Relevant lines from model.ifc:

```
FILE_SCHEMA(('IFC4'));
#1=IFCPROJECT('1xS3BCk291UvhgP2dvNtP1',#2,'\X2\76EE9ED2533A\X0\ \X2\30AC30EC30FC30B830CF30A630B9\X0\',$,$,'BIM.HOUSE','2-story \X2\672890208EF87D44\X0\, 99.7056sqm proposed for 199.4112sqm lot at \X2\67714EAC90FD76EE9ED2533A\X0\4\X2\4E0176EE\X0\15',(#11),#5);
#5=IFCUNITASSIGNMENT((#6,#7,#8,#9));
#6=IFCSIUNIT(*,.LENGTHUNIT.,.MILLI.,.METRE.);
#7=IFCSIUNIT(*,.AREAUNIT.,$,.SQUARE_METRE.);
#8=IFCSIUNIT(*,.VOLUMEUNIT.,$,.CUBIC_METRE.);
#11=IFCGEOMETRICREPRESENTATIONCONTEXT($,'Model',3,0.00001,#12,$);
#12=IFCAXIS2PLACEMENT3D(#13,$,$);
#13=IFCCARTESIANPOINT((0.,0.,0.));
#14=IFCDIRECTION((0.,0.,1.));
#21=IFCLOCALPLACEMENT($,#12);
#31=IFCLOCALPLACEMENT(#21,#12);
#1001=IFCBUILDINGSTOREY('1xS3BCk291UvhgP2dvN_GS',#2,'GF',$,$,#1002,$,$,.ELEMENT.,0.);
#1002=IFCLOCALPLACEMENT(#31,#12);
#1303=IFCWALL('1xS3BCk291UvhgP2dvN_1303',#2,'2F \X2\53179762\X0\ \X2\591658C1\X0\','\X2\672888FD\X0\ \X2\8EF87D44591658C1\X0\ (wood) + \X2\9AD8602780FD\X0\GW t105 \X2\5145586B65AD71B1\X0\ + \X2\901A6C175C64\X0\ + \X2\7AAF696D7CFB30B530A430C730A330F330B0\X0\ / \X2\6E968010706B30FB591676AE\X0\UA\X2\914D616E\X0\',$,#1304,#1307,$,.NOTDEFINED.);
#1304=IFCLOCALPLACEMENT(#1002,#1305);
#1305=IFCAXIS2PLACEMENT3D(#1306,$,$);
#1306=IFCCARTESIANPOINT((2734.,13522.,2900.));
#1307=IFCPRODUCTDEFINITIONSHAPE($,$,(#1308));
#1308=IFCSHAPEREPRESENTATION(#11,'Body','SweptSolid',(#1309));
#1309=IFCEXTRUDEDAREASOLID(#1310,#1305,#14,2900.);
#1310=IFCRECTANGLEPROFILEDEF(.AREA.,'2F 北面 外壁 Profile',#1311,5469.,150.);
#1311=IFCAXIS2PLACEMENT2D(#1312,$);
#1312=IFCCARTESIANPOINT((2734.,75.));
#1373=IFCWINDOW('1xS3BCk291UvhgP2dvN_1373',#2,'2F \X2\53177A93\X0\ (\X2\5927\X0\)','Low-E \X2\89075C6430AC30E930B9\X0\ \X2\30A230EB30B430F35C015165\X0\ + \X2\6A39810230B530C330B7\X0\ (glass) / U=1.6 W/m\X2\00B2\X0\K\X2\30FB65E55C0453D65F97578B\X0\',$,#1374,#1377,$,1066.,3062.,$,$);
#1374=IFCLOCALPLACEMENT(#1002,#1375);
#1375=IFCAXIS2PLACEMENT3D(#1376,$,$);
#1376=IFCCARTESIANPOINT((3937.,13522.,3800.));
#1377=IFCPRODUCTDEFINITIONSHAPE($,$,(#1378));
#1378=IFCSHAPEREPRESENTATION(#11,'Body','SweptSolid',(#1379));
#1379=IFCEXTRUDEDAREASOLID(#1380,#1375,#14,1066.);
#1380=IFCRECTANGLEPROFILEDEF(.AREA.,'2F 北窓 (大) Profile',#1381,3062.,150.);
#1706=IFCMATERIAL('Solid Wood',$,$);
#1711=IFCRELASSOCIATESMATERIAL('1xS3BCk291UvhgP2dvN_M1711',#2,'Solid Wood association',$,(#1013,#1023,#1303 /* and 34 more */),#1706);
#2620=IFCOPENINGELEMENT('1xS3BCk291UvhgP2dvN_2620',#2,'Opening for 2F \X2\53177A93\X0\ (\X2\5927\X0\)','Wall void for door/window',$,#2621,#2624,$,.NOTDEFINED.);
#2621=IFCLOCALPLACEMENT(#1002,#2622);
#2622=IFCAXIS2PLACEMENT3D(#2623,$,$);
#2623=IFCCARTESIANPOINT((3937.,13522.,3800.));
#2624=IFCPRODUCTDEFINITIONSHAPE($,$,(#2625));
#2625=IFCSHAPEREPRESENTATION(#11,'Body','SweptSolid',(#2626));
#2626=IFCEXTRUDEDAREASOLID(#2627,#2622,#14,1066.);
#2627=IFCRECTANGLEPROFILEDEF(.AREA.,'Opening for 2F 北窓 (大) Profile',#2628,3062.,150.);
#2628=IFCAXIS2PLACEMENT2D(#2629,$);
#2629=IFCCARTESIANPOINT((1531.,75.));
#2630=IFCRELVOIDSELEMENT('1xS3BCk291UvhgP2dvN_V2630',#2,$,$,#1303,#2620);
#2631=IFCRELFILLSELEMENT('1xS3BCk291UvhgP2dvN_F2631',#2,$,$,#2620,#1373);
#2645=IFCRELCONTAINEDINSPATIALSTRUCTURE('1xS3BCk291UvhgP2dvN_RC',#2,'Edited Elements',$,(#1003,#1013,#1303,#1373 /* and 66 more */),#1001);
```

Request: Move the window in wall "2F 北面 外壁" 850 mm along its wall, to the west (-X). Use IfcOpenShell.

```python
import ifcopenshell
import ifcopenshell.api.geometry
import ifcopenshell.util.placement
import ifcopenshell.util.unit

model = ifcopenshell.open("model.ifc")
unit_scale = ifcopenshell.util.unit.calculate_unit_scale(model)

window = model.by_guid("1xS3BCk291UvhgP2dvN_1373")
opening = window.FillsVoids[0].RelatingOpeningElement
wall = opening.VoidsElements[0].RelatingBuildingElement

wall_matrix = ifcopenshell.util.placement.get_local_placement(wall.ObjectPlacement)
shift = wall_matrix[:3, 0] * -0.85 / unit_scale
before = ifcopenshell.util.placement.get_local_placement(window.ObjectPlacement)[:3, 3].copy()

# The window is not placed relative to its opening, so move both.
for product in (opening, window):
    matrix = ifcopenshell.util.placement.get_local_placement(product.ObjectPlacement)
    matrix[:3, 3] += shift
    ifcopenshell.api.geometry.edit_object_placement(model, product=product, matrix=matrix, is_si=False)

after = ifcopenshell.util.placement.get_local_placement(window.ObjectPlacement)[:3, 3]
print("window moved by", (after - before).round(3) + 0.0)

model.write("model-out.ifc")
```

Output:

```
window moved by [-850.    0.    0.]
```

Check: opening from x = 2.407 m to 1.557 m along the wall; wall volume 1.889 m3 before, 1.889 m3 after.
